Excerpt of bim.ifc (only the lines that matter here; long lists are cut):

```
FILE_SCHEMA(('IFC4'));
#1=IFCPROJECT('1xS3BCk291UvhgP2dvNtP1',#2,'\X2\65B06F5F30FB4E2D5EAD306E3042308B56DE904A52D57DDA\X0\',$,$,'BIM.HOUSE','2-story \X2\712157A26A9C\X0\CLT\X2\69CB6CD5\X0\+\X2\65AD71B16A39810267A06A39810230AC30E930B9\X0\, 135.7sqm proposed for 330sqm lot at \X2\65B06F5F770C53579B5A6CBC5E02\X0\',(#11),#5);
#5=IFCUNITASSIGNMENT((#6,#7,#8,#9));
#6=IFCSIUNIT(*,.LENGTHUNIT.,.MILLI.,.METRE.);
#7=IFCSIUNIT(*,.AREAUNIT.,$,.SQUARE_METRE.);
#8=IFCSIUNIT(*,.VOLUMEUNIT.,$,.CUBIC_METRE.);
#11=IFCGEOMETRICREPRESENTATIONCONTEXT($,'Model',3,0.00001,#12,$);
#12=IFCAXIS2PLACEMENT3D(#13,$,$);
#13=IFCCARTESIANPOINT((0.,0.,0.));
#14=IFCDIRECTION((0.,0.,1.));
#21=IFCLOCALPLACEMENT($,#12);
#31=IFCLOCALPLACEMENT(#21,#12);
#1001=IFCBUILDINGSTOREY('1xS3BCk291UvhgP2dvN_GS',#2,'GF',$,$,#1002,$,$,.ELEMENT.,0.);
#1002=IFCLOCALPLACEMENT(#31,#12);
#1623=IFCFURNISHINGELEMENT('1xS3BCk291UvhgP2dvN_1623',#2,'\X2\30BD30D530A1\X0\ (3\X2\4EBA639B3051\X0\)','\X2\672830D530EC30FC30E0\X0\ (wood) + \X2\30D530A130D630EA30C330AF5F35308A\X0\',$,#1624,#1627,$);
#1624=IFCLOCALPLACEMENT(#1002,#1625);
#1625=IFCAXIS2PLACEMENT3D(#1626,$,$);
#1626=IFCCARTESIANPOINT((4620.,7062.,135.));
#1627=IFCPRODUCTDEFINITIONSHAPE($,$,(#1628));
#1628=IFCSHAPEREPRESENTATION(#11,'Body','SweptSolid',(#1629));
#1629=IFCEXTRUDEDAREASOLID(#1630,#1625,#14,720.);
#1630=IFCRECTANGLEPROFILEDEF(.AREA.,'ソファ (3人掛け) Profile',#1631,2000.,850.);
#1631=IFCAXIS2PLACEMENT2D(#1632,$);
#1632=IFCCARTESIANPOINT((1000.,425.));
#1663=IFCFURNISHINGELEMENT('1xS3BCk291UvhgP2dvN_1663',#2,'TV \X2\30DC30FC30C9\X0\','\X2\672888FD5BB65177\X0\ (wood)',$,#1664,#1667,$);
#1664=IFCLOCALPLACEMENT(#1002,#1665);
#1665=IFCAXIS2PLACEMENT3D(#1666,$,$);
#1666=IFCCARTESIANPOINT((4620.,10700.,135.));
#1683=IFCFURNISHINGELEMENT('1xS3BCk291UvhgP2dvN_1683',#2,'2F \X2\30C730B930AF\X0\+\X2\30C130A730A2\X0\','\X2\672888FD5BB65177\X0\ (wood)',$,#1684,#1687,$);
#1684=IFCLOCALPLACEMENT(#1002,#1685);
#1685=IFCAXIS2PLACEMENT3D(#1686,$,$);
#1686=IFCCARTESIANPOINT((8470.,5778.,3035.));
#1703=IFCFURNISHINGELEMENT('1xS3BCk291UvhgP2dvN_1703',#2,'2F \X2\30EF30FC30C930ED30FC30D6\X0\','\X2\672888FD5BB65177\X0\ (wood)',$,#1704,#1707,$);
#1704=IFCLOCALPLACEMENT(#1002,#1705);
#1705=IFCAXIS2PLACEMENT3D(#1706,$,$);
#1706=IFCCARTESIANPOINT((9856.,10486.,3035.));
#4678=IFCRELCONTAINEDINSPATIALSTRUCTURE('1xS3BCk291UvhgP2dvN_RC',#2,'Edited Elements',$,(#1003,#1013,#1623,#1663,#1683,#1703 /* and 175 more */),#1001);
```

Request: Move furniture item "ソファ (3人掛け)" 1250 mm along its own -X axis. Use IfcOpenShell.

```python
import ifcopenshell
import ifcopenshell.api.geometry
import ifcopenshell.util.placement
import ifcopenshell.util.unit

model = ifcopenshell.open("bim.ifc")
unit_scale = ifcopenshell.util.unit.calculate_unit_scale(model)

item = model.by_guid("1xS3BCk291UvhgP2dvN_1623")
matrix = ifcopenshell.util.placement.get_local_placement(item.ObjectPlacement)
matrix[:3, 3] -= matrix[:3, 0] * 1.25 / unit_scale
ifcopenshell.api.geometry.edit_object_placement(model, product=item, matrix=matrix, is_si=False)

print(ifcopenshell.util.placement.get_local_placement(item.ObjectPlacement).round(3) + 0.0)

model.write("bim_edited.ifc")
```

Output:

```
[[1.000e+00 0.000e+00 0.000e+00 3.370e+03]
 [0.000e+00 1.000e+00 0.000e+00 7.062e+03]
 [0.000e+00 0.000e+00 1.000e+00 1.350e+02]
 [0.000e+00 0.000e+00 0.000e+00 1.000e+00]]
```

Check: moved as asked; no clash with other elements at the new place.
